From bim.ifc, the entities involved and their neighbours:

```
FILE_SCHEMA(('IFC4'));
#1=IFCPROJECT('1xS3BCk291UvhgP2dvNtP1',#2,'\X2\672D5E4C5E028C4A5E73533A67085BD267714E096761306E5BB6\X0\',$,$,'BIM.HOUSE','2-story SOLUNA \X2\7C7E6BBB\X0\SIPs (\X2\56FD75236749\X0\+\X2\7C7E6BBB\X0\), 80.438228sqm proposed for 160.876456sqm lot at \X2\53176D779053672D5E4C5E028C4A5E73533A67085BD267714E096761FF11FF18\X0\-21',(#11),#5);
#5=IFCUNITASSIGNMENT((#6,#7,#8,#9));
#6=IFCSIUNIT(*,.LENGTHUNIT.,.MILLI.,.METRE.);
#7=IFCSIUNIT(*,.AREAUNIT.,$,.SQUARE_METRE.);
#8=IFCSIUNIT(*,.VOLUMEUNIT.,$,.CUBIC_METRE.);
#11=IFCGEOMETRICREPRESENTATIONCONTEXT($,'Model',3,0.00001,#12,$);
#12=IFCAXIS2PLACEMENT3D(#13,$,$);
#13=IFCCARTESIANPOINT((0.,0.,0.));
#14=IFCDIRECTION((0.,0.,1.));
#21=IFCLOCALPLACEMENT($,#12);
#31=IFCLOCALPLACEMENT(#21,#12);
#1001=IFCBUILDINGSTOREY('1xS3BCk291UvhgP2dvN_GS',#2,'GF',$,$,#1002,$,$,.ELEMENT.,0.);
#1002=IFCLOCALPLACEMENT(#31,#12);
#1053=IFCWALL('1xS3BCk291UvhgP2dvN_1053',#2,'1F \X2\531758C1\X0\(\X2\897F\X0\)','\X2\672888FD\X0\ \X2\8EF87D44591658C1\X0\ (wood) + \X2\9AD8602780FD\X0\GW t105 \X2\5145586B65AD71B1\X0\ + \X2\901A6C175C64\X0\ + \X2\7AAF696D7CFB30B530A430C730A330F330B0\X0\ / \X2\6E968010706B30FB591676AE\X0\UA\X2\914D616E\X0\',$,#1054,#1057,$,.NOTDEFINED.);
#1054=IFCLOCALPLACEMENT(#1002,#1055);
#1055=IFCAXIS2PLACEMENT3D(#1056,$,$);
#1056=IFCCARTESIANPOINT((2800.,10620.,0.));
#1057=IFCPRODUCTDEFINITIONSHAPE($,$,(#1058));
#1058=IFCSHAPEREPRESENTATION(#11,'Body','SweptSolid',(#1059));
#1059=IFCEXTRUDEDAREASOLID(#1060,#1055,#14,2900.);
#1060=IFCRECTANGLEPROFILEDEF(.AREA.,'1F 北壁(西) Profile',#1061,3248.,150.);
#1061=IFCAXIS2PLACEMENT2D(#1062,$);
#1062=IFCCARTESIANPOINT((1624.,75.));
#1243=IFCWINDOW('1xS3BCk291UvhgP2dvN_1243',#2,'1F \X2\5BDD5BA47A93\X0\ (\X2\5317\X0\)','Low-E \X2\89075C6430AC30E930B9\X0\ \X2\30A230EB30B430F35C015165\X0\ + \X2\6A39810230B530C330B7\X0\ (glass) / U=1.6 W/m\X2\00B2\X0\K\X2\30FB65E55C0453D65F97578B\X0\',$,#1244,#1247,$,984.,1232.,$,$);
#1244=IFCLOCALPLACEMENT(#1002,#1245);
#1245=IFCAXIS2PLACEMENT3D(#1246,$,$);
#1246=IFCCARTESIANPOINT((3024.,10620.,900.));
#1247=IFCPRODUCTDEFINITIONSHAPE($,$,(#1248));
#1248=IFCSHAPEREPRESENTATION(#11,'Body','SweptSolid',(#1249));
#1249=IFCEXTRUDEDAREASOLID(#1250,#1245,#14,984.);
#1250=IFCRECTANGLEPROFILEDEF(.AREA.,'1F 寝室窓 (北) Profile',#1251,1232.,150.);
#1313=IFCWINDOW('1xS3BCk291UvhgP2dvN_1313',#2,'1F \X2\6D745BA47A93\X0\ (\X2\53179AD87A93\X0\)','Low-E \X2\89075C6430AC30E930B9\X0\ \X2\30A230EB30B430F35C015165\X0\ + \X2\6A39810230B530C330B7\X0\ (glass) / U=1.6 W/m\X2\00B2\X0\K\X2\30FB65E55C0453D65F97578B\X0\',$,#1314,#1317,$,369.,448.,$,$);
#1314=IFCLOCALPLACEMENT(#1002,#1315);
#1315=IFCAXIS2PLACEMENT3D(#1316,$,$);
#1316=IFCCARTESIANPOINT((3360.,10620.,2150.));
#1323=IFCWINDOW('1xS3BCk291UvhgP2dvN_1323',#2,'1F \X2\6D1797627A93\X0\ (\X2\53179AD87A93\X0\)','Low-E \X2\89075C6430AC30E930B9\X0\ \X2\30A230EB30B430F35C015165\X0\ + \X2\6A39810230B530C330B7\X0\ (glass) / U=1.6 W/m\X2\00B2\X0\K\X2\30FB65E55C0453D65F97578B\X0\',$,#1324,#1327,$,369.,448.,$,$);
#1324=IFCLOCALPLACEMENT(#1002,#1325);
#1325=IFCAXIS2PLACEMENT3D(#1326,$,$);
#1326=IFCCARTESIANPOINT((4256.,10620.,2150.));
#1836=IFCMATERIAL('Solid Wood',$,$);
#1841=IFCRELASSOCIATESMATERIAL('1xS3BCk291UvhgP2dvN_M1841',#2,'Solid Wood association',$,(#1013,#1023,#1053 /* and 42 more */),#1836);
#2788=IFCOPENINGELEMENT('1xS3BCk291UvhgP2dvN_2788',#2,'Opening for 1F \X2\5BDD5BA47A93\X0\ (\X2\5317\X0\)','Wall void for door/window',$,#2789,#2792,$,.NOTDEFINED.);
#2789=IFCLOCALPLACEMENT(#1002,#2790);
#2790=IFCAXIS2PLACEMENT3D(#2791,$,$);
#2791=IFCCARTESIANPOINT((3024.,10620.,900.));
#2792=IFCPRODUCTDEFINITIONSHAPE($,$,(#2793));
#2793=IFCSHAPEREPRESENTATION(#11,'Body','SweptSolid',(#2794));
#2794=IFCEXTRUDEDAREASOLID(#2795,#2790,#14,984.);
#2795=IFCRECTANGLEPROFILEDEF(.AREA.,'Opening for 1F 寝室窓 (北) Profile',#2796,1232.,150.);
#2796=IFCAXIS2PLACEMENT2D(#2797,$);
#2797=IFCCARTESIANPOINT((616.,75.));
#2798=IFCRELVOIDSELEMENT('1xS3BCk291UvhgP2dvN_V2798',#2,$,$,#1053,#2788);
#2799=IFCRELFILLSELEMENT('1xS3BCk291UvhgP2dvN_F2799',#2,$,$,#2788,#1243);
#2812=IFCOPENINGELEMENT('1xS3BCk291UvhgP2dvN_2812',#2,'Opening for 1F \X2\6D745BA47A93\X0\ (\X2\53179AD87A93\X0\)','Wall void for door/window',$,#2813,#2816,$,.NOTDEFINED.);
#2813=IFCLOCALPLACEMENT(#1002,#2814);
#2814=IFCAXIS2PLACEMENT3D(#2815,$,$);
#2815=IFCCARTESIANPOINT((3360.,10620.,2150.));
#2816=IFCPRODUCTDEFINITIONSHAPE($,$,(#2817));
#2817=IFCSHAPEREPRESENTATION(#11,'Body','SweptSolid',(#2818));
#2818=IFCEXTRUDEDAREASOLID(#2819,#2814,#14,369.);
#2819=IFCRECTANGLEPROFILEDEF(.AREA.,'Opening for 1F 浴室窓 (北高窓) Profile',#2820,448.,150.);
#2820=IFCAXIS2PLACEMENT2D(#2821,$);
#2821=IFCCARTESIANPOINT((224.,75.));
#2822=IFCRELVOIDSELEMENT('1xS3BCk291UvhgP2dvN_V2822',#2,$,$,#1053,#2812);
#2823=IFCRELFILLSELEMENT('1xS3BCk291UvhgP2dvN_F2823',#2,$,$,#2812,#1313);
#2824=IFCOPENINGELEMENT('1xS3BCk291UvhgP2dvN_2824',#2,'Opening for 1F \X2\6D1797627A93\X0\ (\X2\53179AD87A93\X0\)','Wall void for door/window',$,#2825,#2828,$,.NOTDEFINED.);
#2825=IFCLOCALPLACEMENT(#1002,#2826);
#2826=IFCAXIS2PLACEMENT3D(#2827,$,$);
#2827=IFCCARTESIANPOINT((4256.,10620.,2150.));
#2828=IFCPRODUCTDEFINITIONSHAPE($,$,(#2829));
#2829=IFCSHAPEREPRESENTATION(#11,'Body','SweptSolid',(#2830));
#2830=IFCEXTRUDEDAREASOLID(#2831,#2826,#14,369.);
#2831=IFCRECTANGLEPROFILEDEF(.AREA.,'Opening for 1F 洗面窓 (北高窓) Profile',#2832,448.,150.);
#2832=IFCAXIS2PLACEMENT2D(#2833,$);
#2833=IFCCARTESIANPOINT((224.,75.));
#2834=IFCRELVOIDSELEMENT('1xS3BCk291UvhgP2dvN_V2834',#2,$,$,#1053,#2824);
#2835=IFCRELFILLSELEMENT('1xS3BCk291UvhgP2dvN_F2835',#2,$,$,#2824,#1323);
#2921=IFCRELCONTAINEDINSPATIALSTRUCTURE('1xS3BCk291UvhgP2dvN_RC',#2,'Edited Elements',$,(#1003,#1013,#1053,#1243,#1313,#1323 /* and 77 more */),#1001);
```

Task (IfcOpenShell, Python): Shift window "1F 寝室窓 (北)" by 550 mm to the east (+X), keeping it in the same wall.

```python
import ifcopenshell
import ifcopenshell.api.geometry
import ifcopenshell.util.placement

model = ifcopenshell.open("bim.ifc")

window = model.by_id(1243)
opening = window.FillsVoids[0].RelatingOpeningElement
wall = opening.VoidsElements[0].RelatingBuildingElement

wall_matrix = ifcopenshell.util.placement.get_local_placement(wall.ObjectPlacement)
shift = wall_matrix[:3, 0] * 550.0
before = ifcopenshell.util.placement.get_local_placement(window.ObjectPlacement)[:3, 3].copy()

# The window is not placed relative to its opening, so move both.
for product in (opening, window):
    matrix = ifcopenshell.util.placement.get_local_placement(product.ObjectPlacement)
    matrix[:3, 3] += shift
    ifcopenshell.api.geometry.edit_object_placement(model, product=product, matrix=matrix, is_si=False)

after = ifcopenshell.util.placement.get_local_placement(window.ObjectPlacement)[:3, 3]
print("window moved by", (after - before).round(3) + 0.0)

model.write("bim_v2.ifc")
```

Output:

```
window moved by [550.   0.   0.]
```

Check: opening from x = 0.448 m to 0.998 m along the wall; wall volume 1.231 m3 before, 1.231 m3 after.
